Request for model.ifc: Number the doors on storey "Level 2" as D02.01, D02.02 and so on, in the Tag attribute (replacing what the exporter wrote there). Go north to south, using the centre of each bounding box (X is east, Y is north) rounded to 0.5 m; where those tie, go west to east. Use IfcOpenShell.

First a look at what the model holds.

```python
import ifcopenshell
import ifcopenshell.util.element
import ifcopenshell.util.placement

model = ifcopenshell.open("model.ifc")
print(model.schema)
storey = next(s for s in model.by_type("IfcBuildingStorey") if s.Name == "Level 2")
doors = [e for e in ifcopenshell.util.element.get_decomposition(storey) if e.is_a("IfcDoor")]
for e in sorted(doors, key=lambda e: e.id()):
    origin = ifcopenshell.util.placement.get_local_placement(e.ObjectPlacement)[:3, 3]
    print(e.id(), e.Tag, e.Name, origin.round(2) + 0.0, sep=" | ")
```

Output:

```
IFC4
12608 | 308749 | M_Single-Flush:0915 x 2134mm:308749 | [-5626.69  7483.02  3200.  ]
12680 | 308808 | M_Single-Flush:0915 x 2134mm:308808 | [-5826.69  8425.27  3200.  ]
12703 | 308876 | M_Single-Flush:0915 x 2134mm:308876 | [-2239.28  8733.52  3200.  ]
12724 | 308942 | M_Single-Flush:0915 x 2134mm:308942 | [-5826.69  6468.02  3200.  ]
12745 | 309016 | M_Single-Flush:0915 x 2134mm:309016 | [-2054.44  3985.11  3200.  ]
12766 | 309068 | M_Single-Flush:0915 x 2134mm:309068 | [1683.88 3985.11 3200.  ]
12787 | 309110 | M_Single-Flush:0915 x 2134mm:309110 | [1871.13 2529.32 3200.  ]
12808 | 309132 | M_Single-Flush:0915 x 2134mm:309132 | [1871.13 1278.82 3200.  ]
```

```python
import ifcopenshell
import ifcopenshell.geom
import ifcopenshell.util.element
import ifcopenshell.util.shape

model = ifcopenshell.open("model.ifc")
settings = ifcopenshell.geom.settings()
settings.set("use-world-coords", True)


def centre(element):
    shape = ifcopenshell.geom.create_shape(settings, element)
    return ifcopenshell.util.shape.get_bbox_centroid(shape.geometry)


storey = next(s for s in model.by_type("IfcBuildingStorey") if s.Name == "Level 2")
doors = [e for e in ifcopenshell.util.element.get_decomposition(storey) if e.is_a("IfcDoor")]

# Insertion points can sit at a corner or the storey origin, so sort by the geometry (in metres).
centres = {e: centre(e) for e in doors}
doors.sort(key=lambda e: (-round(centres[e][1] / 0.5), centres[e][0]))

for i, e in enumerate(doors, start=1):
    number = f"D02.{i:02d}"
    e.Tag = number
    print(e.id(), number)

model.write("model_rev.ifc")
```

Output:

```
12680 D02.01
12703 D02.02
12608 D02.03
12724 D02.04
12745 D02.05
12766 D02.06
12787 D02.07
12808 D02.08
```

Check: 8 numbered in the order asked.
